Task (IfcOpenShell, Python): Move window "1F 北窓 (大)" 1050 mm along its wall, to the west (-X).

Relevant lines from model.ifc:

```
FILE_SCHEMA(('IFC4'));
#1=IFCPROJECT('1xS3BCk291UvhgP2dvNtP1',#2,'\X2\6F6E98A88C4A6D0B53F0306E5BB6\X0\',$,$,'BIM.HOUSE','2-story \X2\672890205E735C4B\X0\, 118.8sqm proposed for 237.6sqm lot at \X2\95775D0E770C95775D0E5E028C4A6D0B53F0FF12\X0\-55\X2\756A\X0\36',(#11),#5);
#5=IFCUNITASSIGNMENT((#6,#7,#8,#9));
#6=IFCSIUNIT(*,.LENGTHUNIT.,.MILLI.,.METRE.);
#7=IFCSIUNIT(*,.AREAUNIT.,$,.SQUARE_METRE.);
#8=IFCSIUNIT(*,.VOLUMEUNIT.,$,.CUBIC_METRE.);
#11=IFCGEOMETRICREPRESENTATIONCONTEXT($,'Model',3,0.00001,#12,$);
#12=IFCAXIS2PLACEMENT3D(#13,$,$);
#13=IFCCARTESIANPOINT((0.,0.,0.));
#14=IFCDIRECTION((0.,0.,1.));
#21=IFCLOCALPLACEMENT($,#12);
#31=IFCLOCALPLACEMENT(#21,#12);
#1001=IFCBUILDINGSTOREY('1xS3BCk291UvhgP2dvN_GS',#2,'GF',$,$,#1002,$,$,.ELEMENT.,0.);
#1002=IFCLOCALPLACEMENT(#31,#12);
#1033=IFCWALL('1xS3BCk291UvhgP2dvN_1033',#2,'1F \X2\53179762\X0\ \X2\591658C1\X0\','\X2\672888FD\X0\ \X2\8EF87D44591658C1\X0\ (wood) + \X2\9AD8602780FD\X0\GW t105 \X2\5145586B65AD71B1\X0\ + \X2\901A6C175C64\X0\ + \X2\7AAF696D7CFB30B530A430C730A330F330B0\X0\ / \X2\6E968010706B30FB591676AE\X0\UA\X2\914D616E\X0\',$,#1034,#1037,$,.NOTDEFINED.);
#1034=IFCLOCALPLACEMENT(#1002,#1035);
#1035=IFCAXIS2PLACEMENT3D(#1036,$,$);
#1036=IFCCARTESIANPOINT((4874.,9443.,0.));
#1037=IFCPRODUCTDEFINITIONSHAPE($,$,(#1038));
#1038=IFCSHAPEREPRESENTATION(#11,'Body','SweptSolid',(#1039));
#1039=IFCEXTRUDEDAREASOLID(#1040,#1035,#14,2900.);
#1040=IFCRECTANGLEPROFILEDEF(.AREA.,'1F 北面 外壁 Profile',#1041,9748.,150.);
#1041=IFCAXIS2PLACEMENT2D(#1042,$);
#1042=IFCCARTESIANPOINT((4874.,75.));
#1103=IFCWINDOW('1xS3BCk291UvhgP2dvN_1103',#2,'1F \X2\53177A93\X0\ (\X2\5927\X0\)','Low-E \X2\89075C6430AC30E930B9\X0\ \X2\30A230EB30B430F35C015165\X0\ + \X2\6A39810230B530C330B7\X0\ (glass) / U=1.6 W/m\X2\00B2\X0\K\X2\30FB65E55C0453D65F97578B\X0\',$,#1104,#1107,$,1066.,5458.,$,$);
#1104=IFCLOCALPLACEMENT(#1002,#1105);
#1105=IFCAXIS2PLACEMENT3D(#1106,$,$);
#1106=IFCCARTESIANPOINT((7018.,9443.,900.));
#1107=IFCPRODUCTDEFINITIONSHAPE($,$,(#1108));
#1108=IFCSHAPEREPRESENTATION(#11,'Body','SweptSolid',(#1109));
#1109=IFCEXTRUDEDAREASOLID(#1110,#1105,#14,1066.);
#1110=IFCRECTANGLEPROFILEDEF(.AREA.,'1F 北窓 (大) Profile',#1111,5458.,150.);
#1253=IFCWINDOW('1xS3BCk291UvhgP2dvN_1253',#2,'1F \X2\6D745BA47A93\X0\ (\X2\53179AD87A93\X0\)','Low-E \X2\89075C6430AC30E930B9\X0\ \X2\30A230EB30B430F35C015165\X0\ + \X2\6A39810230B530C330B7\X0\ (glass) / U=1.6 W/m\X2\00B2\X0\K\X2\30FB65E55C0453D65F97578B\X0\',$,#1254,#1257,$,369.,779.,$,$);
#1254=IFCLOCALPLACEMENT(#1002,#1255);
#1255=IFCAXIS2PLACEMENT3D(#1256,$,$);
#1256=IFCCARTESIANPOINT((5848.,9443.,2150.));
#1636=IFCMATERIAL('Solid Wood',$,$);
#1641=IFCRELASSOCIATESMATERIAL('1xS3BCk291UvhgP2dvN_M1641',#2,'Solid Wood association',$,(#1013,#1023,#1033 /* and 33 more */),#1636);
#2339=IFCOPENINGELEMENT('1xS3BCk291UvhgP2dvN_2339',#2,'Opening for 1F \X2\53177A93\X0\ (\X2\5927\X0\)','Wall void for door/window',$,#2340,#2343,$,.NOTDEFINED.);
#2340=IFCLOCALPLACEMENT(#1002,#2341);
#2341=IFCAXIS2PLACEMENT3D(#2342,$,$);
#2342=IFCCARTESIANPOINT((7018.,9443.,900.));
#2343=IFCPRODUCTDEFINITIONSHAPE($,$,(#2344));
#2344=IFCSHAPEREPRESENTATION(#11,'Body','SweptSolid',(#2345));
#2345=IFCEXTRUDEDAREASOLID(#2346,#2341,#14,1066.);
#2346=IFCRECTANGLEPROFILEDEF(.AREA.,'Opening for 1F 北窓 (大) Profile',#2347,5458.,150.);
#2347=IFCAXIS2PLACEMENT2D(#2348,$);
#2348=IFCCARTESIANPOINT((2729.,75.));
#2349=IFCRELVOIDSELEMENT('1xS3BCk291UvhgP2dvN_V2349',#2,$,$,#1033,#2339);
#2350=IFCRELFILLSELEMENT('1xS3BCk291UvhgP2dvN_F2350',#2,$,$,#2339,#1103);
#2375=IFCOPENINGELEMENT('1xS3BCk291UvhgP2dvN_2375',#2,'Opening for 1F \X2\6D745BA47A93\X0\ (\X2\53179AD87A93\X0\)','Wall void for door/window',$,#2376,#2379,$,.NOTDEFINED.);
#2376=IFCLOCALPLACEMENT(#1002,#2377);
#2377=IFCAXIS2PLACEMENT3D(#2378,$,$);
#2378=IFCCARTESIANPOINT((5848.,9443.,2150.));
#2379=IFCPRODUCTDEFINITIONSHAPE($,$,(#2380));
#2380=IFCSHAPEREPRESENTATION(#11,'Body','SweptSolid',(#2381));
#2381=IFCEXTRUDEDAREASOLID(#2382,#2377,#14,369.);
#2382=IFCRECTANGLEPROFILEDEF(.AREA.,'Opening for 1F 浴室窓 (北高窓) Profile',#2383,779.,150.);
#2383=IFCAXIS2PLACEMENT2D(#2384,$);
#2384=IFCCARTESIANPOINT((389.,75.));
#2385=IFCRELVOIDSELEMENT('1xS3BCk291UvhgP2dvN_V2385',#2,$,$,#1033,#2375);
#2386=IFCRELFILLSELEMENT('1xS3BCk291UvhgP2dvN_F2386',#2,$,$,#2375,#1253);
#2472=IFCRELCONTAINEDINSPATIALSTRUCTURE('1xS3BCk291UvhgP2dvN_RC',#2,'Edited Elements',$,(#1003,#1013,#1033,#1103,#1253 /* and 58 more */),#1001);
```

```python
import ifcopenshell
import ifcopenshell.api.geometry
import ifcopenshell.util.placement
import ifcopenshell.util.unit

model = ifcopenshell.open("model.ifc")
unit_scale = ifcopenshell.util.unit.calculate_unit_scale(model)

window = model.by_guid("1xS3BCk291UvhgP2dvN_1103")
opening = window.FillsVoids[0].RelatingOpeningElement
wall = opening.VoidsElements[0].RelatingBuildingElement

wall_matrix = ifcopenshell.util.placement.get_local_placement(wall.ObjectPlacement)
shift = wall_matrix[:3, 0] * -1.05 / unit_scale
before = ifcopenshell.util.placement.get_local_placement(window.ObjectPlacement)[:3, 3].copy()

# The window is not placed relative to its opening, so move both.
for product in (opening, window):
    matrix = ifcopenshell.util.placement.get_local_placement(product.ObjectPlacement)
    matrix[:3, 3] += shift
    ifcopenshell.api.geometry.edit_object_placement(model, product=product, matrix=matrix, is_si=False)

after = ifcopenshell.util.placement.get_local_placement(window.ObjectPlacement)[:3, 3]
print("window moved by", (after - before).round(3) + 0.0)

model.write("model_edited.ifc")
```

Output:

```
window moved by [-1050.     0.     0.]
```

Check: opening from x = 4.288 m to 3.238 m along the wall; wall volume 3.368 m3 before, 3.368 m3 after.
